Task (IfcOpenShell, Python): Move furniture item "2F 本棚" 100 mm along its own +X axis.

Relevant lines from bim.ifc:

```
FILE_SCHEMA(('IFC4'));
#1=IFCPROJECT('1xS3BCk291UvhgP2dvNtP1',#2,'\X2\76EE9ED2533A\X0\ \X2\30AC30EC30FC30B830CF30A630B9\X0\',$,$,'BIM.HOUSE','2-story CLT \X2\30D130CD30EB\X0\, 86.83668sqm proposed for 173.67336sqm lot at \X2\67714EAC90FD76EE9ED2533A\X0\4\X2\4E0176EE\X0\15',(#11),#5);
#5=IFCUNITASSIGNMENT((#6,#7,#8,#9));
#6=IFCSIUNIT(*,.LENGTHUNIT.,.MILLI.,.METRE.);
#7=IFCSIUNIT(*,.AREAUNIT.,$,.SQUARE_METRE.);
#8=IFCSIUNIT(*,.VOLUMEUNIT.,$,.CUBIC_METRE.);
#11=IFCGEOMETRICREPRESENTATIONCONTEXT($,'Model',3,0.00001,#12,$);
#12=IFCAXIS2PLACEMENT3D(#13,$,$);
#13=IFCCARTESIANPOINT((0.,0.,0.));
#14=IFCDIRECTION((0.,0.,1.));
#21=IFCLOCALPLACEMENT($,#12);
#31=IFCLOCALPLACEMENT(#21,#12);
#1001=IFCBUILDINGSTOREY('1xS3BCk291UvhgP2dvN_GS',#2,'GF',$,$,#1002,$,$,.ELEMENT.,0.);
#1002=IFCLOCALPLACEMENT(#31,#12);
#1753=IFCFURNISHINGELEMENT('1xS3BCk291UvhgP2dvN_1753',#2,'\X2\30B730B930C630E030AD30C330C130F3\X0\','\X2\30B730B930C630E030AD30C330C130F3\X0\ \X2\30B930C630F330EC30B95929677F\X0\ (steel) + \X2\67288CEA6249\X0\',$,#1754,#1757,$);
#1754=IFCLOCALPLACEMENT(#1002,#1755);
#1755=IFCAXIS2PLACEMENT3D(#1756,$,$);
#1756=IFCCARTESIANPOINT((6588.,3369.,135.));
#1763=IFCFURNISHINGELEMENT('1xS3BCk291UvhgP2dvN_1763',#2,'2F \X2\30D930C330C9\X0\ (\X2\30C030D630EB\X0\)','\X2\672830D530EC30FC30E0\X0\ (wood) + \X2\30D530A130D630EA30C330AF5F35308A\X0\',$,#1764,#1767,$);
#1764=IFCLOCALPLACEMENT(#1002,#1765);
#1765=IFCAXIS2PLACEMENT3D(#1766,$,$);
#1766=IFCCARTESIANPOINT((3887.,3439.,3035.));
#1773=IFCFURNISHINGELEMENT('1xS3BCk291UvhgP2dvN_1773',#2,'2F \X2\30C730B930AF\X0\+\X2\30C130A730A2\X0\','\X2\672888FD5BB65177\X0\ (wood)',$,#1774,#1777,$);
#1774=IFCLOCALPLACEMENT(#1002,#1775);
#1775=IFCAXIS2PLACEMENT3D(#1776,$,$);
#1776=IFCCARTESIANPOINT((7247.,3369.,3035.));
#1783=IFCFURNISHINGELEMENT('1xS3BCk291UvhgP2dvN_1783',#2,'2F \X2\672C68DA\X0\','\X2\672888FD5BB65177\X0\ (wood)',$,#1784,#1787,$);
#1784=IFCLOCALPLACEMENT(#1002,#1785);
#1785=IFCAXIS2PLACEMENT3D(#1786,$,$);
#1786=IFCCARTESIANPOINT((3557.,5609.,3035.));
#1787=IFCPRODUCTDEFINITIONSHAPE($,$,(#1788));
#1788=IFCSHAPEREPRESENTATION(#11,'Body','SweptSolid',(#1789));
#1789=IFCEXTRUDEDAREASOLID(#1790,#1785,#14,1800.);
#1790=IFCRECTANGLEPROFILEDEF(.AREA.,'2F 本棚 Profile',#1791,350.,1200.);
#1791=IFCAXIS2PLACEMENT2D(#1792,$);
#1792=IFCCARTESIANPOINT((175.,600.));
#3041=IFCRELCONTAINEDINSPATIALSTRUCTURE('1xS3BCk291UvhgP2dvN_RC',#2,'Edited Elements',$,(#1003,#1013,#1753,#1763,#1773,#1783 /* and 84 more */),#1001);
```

```python
import ifcopenshell
import ifcopenshell.api.geometry
import ifcopenshell.util.placement

model = ifcopenshell.open("bim.ifc")

item = model.by_guid("1xS3BCk291UvhgP2dvN_1783")
matrix = ifcopenshell.util.placement.get_local_placement(item.ObjectPlacement)
matrix[:3, 3] += matrix[:3, 0] * 100.0
ifcopenshell.api.geometry.edit_object_placement(model, product=item, matrix=matrix, is_si=False)

print(ifcopenshell.util.placement.get_local_placement(item.ObjectPlacement).round(3) + 0.0)

model.write("bim_updated.ifc")
```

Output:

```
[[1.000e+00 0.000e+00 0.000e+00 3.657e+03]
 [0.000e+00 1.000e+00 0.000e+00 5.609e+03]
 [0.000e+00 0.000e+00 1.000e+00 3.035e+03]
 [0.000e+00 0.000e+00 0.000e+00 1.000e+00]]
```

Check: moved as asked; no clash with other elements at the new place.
